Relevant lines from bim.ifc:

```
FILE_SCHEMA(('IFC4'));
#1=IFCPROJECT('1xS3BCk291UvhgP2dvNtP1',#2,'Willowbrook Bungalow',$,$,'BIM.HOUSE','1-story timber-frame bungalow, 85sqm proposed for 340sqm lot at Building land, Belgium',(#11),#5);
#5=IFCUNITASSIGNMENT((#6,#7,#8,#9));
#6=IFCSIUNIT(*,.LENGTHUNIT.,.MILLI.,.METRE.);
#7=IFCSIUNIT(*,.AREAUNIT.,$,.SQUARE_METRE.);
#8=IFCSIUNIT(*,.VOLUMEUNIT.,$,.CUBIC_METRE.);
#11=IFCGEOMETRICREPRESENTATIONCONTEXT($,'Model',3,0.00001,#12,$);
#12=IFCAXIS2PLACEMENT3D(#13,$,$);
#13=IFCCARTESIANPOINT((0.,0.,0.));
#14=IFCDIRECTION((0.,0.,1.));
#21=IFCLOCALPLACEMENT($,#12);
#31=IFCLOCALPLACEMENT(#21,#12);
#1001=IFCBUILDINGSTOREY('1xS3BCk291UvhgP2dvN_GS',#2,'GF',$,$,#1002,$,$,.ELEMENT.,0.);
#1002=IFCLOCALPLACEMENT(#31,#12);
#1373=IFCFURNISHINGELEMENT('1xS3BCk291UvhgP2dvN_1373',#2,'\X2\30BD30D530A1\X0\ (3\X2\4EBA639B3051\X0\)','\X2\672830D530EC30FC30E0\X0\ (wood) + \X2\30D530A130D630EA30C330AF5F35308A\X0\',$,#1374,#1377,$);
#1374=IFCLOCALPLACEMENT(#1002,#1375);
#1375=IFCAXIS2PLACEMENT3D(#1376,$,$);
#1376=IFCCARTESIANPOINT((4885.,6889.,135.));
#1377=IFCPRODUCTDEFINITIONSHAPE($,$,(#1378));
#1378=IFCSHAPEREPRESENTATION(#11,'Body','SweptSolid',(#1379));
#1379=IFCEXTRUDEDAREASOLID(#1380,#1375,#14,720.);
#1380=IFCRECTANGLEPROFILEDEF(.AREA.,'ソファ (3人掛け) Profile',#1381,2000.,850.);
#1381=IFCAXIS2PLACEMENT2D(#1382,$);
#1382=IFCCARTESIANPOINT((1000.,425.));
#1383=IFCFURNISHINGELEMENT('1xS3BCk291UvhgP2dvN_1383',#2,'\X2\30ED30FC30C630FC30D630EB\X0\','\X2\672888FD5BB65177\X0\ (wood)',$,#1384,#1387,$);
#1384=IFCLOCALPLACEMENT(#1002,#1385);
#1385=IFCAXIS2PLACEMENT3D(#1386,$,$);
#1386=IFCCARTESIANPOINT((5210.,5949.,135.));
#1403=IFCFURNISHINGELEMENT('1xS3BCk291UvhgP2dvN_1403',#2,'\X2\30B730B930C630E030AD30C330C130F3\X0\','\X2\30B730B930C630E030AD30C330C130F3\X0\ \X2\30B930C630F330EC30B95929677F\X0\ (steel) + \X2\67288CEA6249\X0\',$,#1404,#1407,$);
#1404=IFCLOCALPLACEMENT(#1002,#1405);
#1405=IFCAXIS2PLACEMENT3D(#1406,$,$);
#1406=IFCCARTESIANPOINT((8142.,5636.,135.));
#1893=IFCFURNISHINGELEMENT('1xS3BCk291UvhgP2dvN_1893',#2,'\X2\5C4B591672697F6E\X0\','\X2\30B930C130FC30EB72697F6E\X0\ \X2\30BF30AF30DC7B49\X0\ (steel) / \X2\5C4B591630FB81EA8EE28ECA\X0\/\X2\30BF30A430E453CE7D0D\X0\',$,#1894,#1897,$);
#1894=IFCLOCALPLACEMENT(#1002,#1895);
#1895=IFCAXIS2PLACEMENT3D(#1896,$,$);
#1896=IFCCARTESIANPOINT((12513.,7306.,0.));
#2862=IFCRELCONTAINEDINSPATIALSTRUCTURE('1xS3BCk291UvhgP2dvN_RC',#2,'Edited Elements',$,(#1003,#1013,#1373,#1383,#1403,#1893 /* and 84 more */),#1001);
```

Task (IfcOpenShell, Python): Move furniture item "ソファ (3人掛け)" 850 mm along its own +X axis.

```python
import ifcopenshell
import ifcopenshell.api.geometry
import ifcopenshell.util.placement
import ifcopenshell.util.unit

model = ifcopenshell.open("bim.ifc")
unit_scale = ifcopenshell.util.unit.calculate_unit_scale(model)

item = model.by_id(1373)
matrix = ifcopenshell.util.placement.get_local_placement(item.ObjectPlacement)
matrix[:3, 3] += matrix[:3, 0] * 0.85 / unit_scale
ifcopenshell.api.geometry.edit_object_placement(model, product=item, matrix=matrix, is_si=False)

print(ifcopenshell.util.placement.get_local_placement(item.ObjectPlacement).round(3) + 0.0)

model.write("bim_v2.ifc")
```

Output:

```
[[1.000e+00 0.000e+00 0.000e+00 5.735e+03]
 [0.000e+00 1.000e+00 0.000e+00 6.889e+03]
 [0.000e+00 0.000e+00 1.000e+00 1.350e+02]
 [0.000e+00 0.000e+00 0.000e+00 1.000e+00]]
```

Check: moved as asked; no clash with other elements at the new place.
